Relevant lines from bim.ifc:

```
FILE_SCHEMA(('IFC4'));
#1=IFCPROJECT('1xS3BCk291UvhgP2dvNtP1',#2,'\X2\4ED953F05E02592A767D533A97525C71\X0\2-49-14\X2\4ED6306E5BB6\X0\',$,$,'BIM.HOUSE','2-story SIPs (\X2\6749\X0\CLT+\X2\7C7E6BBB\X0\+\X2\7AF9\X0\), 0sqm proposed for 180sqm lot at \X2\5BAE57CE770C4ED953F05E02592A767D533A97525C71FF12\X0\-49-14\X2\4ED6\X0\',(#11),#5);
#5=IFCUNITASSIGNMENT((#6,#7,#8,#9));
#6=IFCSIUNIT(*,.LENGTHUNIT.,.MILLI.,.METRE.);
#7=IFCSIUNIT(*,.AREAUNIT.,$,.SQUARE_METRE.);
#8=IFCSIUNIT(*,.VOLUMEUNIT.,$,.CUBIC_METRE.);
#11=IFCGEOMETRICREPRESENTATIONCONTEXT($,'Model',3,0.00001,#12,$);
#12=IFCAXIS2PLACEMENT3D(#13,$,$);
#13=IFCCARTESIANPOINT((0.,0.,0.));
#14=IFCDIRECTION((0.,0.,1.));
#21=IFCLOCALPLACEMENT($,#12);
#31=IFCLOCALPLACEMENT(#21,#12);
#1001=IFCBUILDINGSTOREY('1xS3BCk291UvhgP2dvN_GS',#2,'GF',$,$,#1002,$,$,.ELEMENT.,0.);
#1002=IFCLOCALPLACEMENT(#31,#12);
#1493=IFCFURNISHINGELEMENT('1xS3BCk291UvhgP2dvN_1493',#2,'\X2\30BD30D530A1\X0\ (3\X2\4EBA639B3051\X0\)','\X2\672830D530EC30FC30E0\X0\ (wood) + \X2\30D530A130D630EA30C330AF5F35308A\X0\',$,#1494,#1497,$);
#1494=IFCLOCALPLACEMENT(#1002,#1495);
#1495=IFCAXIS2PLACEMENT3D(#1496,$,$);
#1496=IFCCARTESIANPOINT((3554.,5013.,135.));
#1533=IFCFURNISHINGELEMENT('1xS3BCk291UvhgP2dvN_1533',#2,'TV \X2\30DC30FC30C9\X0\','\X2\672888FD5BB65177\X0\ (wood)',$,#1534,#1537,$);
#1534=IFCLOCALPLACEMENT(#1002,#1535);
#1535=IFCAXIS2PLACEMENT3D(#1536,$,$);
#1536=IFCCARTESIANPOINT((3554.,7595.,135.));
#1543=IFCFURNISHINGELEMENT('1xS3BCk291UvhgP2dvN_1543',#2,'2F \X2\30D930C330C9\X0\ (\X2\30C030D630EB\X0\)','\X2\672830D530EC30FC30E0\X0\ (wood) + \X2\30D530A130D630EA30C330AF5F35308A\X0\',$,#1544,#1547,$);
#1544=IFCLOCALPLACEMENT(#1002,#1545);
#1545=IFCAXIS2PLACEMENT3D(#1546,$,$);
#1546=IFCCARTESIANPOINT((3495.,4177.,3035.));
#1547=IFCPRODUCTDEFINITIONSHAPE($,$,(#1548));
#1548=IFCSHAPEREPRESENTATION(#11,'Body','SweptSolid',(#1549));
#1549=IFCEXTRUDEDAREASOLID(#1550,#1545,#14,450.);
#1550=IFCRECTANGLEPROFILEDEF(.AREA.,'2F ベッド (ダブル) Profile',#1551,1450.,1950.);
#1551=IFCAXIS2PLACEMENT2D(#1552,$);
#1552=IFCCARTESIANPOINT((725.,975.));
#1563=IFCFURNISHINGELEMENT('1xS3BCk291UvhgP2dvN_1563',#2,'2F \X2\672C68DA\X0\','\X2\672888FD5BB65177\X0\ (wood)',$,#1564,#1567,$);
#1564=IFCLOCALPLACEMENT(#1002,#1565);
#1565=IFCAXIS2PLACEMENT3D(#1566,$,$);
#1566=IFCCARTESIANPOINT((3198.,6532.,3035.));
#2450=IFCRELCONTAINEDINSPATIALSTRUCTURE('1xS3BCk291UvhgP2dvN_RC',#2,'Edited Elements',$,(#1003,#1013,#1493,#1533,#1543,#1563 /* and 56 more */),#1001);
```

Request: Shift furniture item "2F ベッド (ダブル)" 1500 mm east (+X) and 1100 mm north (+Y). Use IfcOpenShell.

```python
import ifcopenshell
import ifcopenshell.api.geometry
import ifcopenshell.util.placement
import ifcopenshell.util.unit

model = ifcopenshell.open("bim.ifc")
unit_scale = ifcopenshell.util.unit.calculate_unit_scale(model)

item = model.by_guid("1xS3BCk291UvhgP2dvN_1543")
matrix = ifcopenshell.util.placement.get_local_placement(item.ObjectPlacement)
matrix[0, 3] += 1.5 / unit_scale
matrix[1, 3] += 1.1 / unit_scale
ifcopenshell.api.geometry.edit_object_placement(model, product=item, matrix=matrix, is_si=False)

print(ifcopenshell.util.placement.get_local_placement(item.ObjectPlacement).round(3) + 0.0)

model.write("bim_v2.ifc")
```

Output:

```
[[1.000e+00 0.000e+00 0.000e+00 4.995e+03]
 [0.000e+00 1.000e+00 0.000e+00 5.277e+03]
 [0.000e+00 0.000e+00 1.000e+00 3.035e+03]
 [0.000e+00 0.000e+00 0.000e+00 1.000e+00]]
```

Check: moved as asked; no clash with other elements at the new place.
